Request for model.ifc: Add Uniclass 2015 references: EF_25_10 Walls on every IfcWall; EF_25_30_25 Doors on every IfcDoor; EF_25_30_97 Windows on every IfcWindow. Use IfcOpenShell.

First a look at what the model holds.

```python
import ifcopenshell

model = ifcopenshell.open("model.ifc")
print(model.schema)
print("classifications:", [c.Name for c in model.by_type("IfcClassification")])
for ifc_class in ("IfcDoor", "IfcRoof", "IfcStair", "IfcWall", "IfcWindow"):
    print(ifc_class, len(model.by_type(ifc_class)))
```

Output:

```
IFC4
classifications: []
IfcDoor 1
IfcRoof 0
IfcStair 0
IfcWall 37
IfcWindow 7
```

```python
import ifcopenshell
import ifcopenshell.api.classification

model = ifcopenshell.open("model.ifc")

system = ifcopenshell.api.classification.add_classification(model, classification="Uniclass 2015")

codes = {
    "IfcWall": ("EF_25_10", "Walls"),
    "IfcDoor": ("EF_25_30_25", "Doors"),
    "IfcWindow": ("EF_25_30_97", "Windows"),
}
for ifc_class, (code, name) in codes.items():
    products = model.by_type(ifc_class)
    ifcopenshell.api.classification.add_reference(
        model, products=products, classification=system, identification=code, name=name
    )
    print(code, len(products))

model.write("model_v2.ifc")
```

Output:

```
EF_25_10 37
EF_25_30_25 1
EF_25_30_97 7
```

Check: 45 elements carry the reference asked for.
